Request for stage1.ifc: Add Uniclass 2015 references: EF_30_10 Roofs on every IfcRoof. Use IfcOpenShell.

First a look at what the model holds.

```python
import ifcopenshell

model = ifcopenshell.open("stage1.ifc")
print(model.schema)
print("classifications:", [c.Name for c in model.by_type("IfcClassification")])
for ifc_class in ("IfcDoor", "IfcRoof", "IfcStair", "IfcWall", "IfcWindow"):
    print(ifc_class, len(model.by_type(ifc_class)))
```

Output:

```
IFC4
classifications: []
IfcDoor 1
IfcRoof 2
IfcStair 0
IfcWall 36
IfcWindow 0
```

```python
import ifcopenshell
import ifcopenshell.api.classification

model = ifcopenshell.open("stage1.ifc")

system = ifcopenshell.api.classification.add_classification(model, classification="Uniclass 2015")

codes = {
    "IfcRoof": ("EF_30_10", "Roofs"),
}
for ifc_class, (code, name) in codes.items():
    products = model.by_type(ifc_class)
    ifcopenshell.api.classification.add_reference(
        model, products=products, classification=system, identification=code, name=name
    )
    print(code, len(products))

model.write("stage1_edited.ifc")
```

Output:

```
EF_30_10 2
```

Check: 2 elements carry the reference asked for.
